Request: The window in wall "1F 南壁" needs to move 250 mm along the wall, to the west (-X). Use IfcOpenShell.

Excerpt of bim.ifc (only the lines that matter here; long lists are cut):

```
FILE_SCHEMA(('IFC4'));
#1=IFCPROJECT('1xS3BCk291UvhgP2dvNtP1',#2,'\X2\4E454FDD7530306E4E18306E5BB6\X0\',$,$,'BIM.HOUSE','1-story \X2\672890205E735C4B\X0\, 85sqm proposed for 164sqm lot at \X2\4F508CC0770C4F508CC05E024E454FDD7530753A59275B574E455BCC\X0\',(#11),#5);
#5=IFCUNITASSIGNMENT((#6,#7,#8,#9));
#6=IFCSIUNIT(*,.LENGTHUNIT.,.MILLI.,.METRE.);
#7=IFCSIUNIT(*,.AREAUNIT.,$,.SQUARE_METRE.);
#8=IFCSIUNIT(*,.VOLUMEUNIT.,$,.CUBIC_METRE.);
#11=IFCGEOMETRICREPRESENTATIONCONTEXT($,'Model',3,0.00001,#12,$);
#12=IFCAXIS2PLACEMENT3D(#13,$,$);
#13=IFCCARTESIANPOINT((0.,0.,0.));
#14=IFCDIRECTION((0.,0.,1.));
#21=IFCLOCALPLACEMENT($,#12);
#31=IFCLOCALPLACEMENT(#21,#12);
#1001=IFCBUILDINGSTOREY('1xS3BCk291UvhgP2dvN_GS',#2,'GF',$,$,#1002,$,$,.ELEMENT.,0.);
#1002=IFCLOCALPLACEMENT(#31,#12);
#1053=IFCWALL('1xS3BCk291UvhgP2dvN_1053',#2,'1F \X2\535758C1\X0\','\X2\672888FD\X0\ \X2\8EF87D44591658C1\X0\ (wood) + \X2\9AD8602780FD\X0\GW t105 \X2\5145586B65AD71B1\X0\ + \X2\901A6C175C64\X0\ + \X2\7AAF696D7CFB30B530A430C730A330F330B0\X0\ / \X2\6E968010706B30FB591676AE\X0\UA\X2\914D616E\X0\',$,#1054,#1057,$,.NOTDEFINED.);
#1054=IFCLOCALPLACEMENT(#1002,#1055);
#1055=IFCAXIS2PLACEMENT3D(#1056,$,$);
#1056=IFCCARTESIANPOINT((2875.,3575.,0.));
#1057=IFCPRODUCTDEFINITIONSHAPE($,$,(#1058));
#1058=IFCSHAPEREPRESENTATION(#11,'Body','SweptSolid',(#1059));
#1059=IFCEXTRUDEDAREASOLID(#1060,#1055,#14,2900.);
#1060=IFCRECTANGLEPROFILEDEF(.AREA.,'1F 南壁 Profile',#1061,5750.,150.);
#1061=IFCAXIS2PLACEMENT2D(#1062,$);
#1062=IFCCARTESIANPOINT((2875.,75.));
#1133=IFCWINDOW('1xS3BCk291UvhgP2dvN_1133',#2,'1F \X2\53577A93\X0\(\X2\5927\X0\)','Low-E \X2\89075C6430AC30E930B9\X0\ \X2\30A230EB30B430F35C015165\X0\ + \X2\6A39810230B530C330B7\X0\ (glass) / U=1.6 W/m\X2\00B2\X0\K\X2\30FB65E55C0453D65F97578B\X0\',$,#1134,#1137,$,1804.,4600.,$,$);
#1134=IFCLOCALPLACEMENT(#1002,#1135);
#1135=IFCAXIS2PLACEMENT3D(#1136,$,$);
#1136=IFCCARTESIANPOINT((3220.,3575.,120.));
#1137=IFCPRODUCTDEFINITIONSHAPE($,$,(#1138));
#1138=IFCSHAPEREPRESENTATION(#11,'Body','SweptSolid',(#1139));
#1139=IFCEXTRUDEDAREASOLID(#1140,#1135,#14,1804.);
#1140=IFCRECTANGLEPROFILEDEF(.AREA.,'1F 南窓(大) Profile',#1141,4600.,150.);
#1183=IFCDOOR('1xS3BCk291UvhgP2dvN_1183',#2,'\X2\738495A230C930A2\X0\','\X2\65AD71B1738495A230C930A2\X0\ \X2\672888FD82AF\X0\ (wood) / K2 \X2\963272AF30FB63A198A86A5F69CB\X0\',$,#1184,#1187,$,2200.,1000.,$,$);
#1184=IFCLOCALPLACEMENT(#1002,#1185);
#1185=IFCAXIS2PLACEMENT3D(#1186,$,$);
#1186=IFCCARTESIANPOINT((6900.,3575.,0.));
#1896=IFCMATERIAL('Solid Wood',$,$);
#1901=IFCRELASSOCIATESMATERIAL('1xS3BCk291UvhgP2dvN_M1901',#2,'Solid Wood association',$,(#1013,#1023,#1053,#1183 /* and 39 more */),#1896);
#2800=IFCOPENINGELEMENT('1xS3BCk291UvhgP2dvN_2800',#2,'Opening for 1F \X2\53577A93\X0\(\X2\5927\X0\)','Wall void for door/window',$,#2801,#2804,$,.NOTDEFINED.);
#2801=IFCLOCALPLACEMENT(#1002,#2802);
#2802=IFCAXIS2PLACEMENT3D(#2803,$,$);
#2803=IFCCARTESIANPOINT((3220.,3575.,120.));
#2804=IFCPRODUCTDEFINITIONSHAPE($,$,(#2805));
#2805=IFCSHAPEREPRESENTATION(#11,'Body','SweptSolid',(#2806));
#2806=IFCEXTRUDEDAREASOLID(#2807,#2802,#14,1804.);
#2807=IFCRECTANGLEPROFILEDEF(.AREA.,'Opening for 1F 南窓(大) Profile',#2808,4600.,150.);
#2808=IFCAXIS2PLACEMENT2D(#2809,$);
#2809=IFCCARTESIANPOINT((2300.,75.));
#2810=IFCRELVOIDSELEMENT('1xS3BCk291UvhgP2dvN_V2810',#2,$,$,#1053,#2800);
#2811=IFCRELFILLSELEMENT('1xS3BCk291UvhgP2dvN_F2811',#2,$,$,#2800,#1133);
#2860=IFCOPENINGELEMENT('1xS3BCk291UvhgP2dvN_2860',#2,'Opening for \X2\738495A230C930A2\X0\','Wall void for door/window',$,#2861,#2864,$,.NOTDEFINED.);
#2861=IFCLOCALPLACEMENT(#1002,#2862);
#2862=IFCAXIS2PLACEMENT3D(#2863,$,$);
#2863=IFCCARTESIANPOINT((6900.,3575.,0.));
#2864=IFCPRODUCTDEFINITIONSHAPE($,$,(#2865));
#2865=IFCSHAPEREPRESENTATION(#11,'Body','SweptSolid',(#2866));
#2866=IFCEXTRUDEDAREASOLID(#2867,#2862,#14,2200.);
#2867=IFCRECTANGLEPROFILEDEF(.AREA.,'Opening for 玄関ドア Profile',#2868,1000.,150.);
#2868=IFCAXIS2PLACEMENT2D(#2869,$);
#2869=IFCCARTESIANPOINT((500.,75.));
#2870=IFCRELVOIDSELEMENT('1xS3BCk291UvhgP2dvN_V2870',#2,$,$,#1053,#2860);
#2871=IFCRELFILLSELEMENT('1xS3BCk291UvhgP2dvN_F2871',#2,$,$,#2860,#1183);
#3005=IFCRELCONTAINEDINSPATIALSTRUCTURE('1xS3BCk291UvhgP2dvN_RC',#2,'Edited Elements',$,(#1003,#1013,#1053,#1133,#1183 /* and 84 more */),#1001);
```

```python
import ifcopenshell
import ifcopenshell.api.geometry
import ifcopenshell.util.placement

model = ifcopenshell.open("bim.ifc")

window = model.by_id(1133)
opening = window.FillsVoids[0].RelatingOpeningElement
wall = opening.VoidsElements[0].RelatingBuildingElement

wall_matrix = ifcopenshell.util.placement.get_local_placement(wall.ObjectPlacement)
shift = wall_matrix[:3, 0] * -250.0
before = ifcopenshell.util.placement.get_local_placement(window.ObjectPlacement)[:3, 3].copy()

# The window is not placed relative to its opening, so move both.
for product in (opening, window):
    matrix = ifcopenshell.util.placement.get_local_placement(product.ObjectPlacement)
    matrix[:3, 3] += shift
    ifcopenshell.api.geometry.edit_object_placement(model, product=product, matrix=matrix, is_si=False)

after = ifcopenshell.util.placement.get_local_placement(window.ObjectPlacement)[:3, 3]
print("window moved by", (after - before).round(3) + 0.0)

model.write("bim-out.ifc")
```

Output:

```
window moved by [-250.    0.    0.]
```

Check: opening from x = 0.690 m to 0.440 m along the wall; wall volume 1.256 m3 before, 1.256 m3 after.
